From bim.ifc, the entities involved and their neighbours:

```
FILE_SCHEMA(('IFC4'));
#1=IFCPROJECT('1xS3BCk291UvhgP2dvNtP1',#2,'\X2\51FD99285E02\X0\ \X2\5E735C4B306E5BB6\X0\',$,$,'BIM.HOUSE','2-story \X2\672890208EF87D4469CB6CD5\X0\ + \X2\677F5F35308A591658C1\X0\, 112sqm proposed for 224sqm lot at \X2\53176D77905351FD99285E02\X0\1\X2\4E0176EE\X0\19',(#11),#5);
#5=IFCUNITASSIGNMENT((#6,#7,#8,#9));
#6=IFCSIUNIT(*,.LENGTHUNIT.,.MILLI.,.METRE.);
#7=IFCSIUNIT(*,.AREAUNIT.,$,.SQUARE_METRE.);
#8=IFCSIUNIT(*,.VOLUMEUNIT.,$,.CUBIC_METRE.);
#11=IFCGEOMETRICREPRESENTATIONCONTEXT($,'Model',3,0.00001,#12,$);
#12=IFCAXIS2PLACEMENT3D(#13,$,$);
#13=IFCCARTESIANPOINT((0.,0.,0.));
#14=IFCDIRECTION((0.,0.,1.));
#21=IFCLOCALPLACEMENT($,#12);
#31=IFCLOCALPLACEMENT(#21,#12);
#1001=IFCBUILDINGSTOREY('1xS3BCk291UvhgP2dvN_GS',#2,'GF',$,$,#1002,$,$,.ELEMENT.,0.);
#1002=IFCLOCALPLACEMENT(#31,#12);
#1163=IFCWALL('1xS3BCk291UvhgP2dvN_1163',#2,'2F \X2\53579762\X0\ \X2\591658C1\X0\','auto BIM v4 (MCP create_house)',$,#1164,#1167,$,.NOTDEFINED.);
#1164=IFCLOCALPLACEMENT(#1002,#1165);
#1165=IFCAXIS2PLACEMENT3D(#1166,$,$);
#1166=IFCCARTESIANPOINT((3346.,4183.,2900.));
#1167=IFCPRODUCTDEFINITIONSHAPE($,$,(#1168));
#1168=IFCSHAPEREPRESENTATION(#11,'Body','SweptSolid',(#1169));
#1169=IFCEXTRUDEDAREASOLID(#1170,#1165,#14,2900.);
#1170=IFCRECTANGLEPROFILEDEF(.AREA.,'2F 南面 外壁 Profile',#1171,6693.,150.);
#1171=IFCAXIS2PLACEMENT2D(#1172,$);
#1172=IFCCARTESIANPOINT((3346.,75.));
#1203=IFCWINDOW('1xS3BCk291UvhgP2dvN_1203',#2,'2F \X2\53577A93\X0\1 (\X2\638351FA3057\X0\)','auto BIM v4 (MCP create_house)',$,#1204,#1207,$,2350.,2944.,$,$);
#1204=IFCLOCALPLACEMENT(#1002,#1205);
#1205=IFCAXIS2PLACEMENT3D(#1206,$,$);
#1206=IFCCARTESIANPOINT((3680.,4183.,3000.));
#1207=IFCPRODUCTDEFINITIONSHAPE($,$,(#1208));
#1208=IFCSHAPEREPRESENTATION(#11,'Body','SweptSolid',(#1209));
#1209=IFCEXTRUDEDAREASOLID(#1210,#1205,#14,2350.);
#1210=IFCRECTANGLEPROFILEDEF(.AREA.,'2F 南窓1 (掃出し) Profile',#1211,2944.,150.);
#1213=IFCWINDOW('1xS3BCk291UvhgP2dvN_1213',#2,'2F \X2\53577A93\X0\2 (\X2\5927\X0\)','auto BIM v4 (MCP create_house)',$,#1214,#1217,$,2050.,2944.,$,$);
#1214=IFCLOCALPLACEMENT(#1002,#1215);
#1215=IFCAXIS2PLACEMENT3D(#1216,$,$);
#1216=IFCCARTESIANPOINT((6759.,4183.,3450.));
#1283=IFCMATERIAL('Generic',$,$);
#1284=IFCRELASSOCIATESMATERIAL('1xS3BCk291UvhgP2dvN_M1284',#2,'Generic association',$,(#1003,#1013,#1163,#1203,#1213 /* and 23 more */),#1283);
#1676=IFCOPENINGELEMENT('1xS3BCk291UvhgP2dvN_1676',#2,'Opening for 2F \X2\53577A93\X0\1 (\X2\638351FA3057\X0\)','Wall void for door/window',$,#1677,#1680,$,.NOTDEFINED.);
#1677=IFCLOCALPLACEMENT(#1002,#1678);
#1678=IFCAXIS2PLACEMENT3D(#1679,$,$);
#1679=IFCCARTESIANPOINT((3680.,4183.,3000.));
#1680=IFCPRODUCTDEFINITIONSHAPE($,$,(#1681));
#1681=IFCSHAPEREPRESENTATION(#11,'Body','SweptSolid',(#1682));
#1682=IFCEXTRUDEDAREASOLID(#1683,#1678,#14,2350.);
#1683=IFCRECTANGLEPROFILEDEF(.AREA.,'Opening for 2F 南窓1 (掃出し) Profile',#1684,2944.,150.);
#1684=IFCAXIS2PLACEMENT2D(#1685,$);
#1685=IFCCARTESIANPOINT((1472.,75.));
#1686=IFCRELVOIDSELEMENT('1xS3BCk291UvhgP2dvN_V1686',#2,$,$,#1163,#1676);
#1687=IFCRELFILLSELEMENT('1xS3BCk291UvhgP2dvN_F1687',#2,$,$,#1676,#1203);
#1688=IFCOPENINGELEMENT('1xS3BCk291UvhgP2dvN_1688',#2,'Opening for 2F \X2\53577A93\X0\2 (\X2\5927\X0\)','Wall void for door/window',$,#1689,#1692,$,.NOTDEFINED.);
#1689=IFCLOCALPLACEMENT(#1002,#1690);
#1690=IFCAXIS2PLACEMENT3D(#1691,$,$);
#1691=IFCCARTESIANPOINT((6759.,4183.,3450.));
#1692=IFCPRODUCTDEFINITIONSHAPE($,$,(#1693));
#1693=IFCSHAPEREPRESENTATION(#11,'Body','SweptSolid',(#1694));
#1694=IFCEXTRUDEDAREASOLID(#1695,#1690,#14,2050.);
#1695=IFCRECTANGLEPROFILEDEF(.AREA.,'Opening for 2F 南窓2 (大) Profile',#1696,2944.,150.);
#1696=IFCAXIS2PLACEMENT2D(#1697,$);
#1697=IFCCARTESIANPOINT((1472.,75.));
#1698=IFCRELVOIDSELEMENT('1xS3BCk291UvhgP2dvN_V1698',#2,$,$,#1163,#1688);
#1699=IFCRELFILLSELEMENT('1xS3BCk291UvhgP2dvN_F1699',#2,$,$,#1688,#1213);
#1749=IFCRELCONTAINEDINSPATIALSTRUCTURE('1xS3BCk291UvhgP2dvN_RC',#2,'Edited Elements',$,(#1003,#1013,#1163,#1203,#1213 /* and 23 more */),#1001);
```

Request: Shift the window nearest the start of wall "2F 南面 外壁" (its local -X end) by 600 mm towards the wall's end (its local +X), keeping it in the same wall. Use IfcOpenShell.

```python
import ifcopenshell
import ifcopenshell.api.geometry
import ifcopenshell.util.placement

model = ifcopenshell.open("bim.ifc")

window = model.by_guid("1xS3BCk291UvhgP2dvN_1203")
opening = window.FillsVoids[0].RelatingOpeningElement
wall = opening.VoidsElements[0].RelatingBuildingElement

wall_matrix = ifcopenshell.util.placement.get_local_placement(wall.ObjectPlacement)
shift = wall_matrix[:3, 0] * 600.0
before = ifcopenshell.util.placement.get_local_placement(window.ObjectPlacement)[:3, 3].copy()

# The window is not placed relative to its opening, so move both.
for product in (opening, window):
    matrix = ifcopenshell.util.placement.get_local_placement(product.ObjectPlacement)
    matrix[:3, 3] += shift
    ifcopenshell.api.geometry.edit_object_placement(model, product=product, matrix=matrix, is_si=False)

after = ifcopenshell.util.placement.get_local_placement(window.ObjectPlacement)[:3, 3]
print("window moved by", (after - before).round(3) + 0.0)

model.write("bim-out.ifc")
```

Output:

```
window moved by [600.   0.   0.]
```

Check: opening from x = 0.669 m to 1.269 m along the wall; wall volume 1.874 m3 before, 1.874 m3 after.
